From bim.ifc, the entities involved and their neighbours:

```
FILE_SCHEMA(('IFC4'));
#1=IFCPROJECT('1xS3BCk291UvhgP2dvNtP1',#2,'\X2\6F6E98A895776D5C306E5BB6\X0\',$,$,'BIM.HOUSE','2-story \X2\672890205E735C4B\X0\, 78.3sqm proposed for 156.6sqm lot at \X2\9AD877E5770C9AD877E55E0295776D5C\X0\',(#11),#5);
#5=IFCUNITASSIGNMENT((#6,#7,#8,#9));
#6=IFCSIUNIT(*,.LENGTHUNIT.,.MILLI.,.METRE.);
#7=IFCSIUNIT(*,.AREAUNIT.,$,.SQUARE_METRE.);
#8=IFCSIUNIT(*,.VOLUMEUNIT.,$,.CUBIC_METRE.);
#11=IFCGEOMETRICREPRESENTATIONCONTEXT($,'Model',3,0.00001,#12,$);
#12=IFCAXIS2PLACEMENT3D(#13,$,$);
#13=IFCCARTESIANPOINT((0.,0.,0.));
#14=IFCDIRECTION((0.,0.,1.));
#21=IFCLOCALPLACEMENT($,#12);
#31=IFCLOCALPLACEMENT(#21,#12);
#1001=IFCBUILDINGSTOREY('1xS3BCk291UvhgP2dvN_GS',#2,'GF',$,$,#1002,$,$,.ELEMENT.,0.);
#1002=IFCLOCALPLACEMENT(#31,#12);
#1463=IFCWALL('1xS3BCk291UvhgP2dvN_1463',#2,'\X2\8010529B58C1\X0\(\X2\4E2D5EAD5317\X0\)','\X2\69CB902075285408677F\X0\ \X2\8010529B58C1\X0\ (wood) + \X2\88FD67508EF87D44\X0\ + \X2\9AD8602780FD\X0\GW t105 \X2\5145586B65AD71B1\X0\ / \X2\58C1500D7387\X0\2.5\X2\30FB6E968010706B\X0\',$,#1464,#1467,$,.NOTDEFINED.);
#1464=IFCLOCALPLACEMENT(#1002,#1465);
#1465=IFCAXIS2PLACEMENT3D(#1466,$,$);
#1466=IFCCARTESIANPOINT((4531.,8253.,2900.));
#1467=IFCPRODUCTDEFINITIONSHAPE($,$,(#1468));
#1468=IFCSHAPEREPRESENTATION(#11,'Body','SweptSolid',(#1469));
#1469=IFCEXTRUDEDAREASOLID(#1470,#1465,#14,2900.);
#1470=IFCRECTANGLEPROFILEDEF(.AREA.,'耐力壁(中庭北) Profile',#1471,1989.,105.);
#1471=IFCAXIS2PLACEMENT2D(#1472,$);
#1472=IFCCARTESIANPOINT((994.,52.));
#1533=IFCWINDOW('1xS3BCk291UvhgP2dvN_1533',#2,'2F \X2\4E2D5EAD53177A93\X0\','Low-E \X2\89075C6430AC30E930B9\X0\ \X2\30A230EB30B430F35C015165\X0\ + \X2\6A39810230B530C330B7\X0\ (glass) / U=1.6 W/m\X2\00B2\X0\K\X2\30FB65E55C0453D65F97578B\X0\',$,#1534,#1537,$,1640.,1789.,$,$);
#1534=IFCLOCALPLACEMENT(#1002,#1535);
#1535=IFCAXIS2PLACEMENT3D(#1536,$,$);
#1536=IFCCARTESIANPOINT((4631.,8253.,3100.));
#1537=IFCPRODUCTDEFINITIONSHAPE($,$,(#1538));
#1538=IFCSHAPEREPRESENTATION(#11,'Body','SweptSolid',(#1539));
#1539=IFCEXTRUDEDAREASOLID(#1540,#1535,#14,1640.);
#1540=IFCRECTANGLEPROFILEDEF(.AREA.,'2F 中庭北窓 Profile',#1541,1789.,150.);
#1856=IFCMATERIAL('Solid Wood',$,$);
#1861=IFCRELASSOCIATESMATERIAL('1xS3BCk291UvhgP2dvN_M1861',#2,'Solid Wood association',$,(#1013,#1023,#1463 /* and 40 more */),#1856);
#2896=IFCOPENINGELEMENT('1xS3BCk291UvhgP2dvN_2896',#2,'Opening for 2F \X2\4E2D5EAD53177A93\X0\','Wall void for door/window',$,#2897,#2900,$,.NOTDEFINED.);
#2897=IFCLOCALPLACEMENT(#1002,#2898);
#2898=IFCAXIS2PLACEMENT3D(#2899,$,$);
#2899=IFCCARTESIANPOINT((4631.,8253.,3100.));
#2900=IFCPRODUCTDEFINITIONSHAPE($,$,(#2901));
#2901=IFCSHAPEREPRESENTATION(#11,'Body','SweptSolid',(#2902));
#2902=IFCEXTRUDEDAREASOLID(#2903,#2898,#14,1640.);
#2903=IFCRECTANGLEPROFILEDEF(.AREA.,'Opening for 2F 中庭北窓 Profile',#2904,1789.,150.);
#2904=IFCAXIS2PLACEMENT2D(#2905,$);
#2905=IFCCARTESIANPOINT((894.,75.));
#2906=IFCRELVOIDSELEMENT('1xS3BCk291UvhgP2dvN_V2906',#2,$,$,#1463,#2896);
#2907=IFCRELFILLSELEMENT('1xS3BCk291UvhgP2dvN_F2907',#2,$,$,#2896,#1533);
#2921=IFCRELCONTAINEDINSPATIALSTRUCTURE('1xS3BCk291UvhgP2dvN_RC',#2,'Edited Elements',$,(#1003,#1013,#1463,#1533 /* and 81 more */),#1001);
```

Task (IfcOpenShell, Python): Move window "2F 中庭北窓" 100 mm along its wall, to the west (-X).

```python
import ifcopenshell
import ifcopenshell.api.geometry
import ifcopenshell.util.placement
import ifcopenshell.util.unit

model = ifcopenshell.open("bim.ifc")
unit_scale = ifcopenshell.util.unit.calculate_unit_scale(model)

window = model.by_guid("1xS3BCk291UvhgP2dvN_1533")
opening = window.FillsVoids[0].RelatingOpeningElement
wall = opening.VoidsElements[0].RelatingBuildingElement

wall_matrix = ifcopenshell.util.placement.get_local_placement(wall.ObjectPlacement)
shift = wall_matrix[:3, 0] * -0.1 / unit_scale
before = ifcopenshell.util.placement.get_local_placement(window.ObjectPlacement)[:3, 3].copy()

# The window is not placed relative to its opening, so move both.
for product in (opening, window):
    matrix = ifcopenshell.util.placement.get_local_placement(product.ObjectPlacement)
    matrix[:3, 3] += shift
    ifcopenshell.api.geometry.edit_object_placement(model, product=product, matrix=matrix, is_si=False)

after = ifcopenshell.util.placement.get_local_placement(window.ObjectPlacement)[:3, 3]
print("window moved by", (after - before).round(3) + 0.0)

model.write("bim_updated.ifc")
```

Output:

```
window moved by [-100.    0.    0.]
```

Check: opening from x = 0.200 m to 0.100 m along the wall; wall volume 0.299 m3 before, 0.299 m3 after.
